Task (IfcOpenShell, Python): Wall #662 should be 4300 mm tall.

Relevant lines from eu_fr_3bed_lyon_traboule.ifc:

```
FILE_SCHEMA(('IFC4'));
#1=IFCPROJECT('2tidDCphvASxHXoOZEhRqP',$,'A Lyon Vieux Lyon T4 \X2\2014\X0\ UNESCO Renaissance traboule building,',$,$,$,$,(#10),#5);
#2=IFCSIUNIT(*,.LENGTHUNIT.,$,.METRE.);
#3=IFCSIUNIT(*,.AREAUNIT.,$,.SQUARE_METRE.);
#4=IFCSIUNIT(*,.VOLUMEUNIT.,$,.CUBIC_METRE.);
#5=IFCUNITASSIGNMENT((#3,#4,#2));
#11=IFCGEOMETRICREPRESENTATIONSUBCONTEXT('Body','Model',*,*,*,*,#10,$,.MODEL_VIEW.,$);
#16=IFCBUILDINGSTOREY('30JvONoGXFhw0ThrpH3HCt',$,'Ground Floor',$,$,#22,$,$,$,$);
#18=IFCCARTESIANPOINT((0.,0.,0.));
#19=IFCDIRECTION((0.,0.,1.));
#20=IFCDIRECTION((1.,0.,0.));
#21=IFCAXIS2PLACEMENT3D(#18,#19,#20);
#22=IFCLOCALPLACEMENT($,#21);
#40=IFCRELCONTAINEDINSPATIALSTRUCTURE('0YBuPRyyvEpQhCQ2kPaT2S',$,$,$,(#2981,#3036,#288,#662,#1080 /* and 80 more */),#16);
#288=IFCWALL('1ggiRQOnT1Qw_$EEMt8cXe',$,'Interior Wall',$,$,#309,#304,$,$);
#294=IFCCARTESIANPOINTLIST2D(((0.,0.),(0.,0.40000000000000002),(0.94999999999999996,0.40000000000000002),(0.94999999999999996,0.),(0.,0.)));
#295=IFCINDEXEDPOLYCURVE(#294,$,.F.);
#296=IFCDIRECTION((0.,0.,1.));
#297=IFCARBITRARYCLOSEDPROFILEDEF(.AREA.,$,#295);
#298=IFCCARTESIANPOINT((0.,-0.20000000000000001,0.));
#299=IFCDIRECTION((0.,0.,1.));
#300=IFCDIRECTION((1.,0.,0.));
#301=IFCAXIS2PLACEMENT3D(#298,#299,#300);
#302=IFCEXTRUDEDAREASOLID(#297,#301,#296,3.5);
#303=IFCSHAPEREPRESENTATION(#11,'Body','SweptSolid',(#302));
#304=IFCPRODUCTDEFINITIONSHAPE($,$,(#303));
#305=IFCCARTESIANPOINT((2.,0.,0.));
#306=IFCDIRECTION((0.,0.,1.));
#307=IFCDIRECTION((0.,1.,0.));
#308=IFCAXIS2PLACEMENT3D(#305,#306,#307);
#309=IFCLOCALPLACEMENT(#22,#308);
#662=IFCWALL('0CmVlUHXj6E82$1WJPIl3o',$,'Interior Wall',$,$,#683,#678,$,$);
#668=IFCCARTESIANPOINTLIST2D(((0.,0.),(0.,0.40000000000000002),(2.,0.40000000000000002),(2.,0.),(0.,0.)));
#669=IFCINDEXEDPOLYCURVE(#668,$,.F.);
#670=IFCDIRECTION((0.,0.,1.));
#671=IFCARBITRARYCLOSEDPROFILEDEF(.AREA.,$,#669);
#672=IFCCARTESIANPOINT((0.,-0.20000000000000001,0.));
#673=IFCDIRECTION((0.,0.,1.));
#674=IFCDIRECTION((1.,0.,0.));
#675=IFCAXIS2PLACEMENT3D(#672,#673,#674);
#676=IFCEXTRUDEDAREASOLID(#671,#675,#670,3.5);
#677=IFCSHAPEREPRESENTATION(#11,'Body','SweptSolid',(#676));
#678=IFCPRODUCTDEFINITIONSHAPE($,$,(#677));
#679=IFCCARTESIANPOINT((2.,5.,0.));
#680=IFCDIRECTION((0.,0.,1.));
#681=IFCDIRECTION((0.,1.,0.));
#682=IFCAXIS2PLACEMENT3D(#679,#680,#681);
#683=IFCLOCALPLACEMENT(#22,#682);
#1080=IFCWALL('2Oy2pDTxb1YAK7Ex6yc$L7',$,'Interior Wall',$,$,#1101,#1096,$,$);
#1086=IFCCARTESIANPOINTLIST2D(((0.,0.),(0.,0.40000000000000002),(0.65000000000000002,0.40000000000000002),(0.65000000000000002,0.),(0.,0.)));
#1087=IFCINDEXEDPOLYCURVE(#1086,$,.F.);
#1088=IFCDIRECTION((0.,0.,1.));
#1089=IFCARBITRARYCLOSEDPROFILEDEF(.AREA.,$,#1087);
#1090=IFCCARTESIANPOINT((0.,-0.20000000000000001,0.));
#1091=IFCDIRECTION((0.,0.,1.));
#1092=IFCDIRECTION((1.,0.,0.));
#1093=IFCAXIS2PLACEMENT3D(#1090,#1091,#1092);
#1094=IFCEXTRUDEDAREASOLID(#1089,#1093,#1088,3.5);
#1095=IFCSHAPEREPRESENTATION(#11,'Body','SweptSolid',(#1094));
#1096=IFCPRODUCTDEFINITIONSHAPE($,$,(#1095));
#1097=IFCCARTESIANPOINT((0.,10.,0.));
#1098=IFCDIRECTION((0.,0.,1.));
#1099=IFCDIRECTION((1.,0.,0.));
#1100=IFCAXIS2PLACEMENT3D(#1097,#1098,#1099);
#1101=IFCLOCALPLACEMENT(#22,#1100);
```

```python
import ifcopenshell
import ifcopenshell.geom
import ifcopenshell.util.representation
import ifcopenshell.util.shape

model = ifcopenshell.open("eu_fr_3bed_lyon_traboule.ifc")
settings = ifcopenshell.geom.settings()


def volume(element):
    """Net volume in cubic metres, openings subtracted."""
    shape = ifcopenshell.geom.create_shape(settings, element)
    return ifcopenshell.util.shape.get_volume(shape.geometry)


wall = model.by_guid("0CmVlUHXj6E82$1WJPIl3o")
before = volume(wall)

body = ifcopenshell.util.representation.get_representation(wall, "Model", "Body")
solid = body.Items[0]
old_height = solid.Depth
solid.Depth = 4.3
after = volume(wall)

print(f"height {old_height:g} -> {solid.Depth:g}, volume {before:.3f} -> {after:.3f} m3")

model.write("eu_fr_3bed_lyon_traboule-out.ifc")
```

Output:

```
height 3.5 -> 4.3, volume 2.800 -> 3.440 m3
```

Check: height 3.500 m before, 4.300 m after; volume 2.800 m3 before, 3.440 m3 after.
